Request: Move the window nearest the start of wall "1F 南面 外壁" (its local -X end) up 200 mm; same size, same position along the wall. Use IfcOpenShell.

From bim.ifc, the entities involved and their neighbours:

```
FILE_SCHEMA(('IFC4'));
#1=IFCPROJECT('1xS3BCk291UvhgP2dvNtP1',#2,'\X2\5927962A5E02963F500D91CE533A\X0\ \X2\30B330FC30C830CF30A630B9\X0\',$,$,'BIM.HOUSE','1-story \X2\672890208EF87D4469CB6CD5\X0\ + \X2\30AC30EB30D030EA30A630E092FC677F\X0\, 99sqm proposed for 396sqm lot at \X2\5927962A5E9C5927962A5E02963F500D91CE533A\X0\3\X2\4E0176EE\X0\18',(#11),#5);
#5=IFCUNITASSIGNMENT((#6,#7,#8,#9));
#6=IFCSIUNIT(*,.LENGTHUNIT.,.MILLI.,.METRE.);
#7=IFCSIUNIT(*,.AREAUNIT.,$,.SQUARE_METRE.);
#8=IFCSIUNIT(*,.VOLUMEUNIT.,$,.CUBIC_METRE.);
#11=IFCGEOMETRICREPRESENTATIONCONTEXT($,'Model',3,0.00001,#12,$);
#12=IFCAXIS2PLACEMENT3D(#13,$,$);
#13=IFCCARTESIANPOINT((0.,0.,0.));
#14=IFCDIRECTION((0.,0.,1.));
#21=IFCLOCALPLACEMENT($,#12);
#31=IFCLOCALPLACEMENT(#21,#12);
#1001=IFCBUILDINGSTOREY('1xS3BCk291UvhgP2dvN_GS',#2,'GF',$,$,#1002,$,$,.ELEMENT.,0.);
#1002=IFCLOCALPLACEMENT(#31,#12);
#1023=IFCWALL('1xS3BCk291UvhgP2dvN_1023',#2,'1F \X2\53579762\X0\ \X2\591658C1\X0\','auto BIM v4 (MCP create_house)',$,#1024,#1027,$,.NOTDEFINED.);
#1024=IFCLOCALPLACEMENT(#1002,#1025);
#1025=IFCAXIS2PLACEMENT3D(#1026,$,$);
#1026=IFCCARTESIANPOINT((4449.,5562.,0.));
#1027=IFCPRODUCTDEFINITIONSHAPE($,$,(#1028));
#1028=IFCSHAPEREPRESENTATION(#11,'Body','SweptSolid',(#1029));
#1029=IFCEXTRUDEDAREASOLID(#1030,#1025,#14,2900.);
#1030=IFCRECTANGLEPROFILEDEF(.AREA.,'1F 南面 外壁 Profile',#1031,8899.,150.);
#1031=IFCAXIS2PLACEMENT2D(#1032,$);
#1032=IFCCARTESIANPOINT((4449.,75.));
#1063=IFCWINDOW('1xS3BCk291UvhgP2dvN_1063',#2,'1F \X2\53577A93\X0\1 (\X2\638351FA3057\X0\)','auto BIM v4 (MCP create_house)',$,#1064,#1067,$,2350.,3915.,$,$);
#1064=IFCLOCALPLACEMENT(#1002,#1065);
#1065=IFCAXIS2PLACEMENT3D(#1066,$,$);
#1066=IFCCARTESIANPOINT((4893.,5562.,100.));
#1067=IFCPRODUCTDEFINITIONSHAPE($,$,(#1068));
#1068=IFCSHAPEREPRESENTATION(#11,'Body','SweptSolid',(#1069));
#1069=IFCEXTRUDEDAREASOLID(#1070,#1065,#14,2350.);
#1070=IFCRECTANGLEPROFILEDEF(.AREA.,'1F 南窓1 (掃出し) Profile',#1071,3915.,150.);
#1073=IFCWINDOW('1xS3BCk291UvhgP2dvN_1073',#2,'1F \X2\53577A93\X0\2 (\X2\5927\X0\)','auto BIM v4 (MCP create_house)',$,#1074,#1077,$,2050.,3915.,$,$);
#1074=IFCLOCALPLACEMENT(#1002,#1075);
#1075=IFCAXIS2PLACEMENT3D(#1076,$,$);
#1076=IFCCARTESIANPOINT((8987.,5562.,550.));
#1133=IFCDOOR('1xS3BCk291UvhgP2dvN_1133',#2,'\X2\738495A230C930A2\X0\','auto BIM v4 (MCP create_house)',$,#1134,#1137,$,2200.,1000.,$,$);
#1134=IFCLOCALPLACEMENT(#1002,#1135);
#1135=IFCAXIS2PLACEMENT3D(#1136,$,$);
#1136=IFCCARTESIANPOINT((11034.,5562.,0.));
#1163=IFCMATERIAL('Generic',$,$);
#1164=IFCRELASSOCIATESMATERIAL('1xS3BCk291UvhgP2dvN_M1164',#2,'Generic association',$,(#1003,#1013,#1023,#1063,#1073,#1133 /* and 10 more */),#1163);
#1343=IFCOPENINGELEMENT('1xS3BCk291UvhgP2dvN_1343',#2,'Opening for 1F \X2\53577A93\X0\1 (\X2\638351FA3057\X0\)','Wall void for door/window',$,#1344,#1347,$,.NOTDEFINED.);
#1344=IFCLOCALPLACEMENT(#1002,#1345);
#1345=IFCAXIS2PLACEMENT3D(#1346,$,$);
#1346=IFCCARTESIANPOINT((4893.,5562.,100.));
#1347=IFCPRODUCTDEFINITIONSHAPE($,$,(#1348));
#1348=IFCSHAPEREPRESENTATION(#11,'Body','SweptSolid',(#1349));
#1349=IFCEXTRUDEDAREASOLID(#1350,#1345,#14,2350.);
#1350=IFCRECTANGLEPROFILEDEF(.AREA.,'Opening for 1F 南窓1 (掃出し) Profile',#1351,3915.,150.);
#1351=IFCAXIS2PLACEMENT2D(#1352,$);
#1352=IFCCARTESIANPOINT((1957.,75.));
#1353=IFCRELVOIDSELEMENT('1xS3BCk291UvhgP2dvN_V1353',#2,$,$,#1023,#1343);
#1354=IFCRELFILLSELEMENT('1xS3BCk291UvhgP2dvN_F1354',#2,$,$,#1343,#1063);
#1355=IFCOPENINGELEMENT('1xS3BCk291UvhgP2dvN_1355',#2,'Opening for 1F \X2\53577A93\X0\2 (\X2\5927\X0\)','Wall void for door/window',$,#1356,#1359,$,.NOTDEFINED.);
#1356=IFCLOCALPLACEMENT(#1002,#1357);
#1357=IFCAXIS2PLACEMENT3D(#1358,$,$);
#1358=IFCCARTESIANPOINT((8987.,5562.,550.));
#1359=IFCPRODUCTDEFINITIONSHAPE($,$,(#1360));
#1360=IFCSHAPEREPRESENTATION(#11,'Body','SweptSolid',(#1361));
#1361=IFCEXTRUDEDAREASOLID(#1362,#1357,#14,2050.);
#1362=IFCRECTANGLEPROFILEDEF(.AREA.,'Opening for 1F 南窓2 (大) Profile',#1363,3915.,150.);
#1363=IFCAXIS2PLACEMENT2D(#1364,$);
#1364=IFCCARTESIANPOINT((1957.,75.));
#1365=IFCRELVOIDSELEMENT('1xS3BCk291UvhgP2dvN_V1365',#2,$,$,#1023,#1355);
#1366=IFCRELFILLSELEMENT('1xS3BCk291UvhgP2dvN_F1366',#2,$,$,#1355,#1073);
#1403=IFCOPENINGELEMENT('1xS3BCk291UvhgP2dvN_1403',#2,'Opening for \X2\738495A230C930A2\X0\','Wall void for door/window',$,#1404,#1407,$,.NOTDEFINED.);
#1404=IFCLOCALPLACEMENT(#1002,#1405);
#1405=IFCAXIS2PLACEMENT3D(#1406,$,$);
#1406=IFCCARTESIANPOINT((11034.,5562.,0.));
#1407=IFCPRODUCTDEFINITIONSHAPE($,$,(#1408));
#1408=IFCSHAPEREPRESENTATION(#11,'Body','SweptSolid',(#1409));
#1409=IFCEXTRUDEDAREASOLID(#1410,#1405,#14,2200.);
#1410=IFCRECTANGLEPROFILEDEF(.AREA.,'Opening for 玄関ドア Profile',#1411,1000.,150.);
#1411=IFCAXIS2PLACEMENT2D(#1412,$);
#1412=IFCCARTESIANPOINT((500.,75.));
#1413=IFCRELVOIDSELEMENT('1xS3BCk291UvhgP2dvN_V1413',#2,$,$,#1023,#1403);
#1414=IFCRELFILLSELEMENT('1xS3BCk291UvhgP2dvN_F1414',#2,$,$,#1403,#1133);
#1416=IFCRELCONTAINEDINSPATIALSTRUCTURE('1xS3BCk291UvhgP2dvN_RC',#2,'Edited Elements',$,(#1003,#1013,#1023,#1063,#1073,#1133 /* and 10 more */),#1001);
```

```python
import numpy as np
import ifcopenshell
import ifcopenshell.api.geometry
import ifcopenshell.util.placement
import ifcopenshell.util.unit

model = ifcopenshell.open("bim.ifc")
unit_scale = ifcopenshell.util.unit.calculate_unit_scale(model)

window = model.by_guid("1xS3BCk291UvhgP2dvN_1063")
opening = window.FillsVoids[0].RelatingOpeningElement
dz = 200.0

shift = np.array([0.0, 0.0, dz])
# The window is not placed relative to its opening, so move both.
for product in (opening, window):
    matrix = ifcopenshell.util.placement.get_local_placement(product.ObjectPlacement)
    matrix[:3, 3] += shift
    ifcopenshell.api.geometry.edit_object_placement(model, product=product, matrix=matrix, is_si=False)

print(f"moved by {dz * unit_scale:+.3f} m")

model.write("bim-out.ifc")
```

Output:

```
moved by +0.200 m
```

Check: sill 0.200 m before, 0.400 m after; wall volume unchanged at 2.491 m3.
